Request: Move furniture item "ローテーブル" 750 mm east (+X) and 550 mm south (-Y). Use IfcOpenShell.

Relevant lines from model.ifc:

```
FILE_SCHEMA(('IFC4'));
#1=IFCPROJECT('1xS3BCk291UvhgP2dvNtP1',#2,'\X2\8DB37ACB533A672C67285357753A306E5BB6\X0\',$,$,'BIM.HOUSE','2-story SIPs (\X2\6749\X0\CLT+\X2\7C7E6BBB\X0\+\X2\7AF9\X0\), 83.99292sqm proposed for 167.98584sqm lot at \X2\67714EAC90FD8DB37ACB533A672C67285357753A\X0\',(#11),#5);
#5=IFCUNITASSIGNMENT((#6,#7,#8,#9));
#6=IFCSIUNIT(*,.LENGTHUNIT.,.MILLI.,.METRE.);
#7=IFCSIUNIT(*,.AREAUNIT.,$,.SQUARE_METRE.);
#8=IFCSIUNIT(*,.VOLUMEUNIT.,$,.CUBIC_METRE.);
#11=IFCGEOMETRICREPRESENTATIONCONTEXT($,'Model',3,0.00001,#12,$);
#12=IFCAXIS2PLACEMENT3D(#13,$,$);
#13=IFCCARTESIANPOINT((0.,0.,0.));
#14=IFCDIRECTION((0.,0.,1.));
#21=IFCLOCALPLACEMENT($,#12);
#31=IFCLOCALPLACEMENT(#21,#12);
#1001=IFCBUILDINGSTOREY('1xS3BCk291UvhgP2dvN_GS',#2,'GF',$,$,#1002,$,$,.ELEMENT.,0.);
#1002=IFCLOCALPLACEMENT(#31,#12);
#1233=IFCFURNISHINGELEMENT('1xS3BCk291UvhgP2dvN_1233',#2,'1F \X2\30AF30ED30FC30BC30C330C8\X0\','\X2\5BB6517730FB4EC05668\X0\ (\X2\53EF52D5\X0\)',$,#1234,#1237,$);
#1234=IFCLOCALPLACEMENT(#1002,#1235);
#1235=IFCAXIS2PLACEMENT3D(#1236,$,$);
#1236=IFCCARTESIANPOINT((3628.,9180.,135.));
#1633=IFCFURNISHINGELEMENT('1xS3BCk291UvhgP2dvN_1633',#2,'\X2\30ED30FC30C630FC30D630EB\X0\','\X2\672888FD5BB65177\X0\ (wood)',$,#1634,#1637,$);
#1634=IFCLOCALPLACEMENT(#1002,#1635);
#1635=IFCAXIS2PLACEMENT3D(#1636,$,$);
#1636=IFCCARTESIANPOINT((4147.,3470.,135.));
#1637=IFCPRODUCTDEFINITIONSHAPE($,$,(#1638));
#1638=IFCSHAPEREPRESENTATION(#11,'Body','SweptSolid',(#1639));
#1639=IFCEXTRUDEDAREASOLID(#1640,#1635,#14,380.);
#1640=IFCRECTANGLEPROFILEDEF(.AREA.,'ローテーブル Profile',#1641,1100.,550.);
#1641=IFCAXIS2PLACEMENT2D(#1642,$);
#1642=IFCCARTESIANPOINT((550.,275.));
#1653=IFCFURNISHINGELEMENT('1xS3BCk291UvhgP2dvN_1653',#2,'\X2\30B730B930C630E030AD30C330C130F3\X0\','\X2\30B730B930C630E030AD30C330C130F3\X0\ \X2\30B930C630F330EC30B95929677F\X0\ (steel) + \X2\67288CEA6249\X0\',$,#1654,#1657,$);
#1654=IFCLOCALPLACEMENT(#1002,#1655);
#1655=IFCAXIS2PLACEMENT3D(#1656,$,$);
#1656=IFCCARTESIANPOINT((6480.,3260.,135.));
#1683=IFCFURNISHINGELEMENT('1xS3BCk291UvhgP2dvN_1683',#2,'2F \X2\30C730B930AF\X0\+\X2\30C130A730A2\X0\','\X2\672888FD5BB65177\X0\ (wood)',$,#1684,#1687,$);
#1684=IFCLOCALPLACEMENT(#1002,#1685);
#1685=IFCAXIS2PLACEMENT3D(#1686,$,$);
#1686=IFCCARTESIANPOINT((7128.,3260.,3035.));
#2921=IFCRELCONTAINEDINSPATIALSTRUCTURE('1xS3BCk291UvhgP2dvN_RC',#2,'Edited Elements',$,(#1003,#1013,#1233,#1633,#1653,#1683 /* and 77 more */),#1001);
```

```python
import ifcopenshell
import ifcopenshell.api.geometry
import ifcopenshell.util.placement
import ifcopenshell.util.unit

model = ifcopenshell.open("model.ifc")
unit_scale = ifcopenshell.util.unit.calculate_unit_scale(model)

item = model.by_guid("1xS3BCk291UvhgP2dvN_1633")
matrix = ifcopenshell.util.placement.get_local_placement(item.ObjectPlacement)
matrix[0, 3] += 0.75 / unit_scale
matrix[1, 3] -= 0.55 / unit_scale
ifcopenshell.api.geometry.edit_object_placement(model, product=item, matrix=matrix, is_si=False)

print(ifcopenshell.util.placement.get_local_placement(item.ObjectPlacement).round(3) + 0.0)

model.write("model_updated.ifc")
```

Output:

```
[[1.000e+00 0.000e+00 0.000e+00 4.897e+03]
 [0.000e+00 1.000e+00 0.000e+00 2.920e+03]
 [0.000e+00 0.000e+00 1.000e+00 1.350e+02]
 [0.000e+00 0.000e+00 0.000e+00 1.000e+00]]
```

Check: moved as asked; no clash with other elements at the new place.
